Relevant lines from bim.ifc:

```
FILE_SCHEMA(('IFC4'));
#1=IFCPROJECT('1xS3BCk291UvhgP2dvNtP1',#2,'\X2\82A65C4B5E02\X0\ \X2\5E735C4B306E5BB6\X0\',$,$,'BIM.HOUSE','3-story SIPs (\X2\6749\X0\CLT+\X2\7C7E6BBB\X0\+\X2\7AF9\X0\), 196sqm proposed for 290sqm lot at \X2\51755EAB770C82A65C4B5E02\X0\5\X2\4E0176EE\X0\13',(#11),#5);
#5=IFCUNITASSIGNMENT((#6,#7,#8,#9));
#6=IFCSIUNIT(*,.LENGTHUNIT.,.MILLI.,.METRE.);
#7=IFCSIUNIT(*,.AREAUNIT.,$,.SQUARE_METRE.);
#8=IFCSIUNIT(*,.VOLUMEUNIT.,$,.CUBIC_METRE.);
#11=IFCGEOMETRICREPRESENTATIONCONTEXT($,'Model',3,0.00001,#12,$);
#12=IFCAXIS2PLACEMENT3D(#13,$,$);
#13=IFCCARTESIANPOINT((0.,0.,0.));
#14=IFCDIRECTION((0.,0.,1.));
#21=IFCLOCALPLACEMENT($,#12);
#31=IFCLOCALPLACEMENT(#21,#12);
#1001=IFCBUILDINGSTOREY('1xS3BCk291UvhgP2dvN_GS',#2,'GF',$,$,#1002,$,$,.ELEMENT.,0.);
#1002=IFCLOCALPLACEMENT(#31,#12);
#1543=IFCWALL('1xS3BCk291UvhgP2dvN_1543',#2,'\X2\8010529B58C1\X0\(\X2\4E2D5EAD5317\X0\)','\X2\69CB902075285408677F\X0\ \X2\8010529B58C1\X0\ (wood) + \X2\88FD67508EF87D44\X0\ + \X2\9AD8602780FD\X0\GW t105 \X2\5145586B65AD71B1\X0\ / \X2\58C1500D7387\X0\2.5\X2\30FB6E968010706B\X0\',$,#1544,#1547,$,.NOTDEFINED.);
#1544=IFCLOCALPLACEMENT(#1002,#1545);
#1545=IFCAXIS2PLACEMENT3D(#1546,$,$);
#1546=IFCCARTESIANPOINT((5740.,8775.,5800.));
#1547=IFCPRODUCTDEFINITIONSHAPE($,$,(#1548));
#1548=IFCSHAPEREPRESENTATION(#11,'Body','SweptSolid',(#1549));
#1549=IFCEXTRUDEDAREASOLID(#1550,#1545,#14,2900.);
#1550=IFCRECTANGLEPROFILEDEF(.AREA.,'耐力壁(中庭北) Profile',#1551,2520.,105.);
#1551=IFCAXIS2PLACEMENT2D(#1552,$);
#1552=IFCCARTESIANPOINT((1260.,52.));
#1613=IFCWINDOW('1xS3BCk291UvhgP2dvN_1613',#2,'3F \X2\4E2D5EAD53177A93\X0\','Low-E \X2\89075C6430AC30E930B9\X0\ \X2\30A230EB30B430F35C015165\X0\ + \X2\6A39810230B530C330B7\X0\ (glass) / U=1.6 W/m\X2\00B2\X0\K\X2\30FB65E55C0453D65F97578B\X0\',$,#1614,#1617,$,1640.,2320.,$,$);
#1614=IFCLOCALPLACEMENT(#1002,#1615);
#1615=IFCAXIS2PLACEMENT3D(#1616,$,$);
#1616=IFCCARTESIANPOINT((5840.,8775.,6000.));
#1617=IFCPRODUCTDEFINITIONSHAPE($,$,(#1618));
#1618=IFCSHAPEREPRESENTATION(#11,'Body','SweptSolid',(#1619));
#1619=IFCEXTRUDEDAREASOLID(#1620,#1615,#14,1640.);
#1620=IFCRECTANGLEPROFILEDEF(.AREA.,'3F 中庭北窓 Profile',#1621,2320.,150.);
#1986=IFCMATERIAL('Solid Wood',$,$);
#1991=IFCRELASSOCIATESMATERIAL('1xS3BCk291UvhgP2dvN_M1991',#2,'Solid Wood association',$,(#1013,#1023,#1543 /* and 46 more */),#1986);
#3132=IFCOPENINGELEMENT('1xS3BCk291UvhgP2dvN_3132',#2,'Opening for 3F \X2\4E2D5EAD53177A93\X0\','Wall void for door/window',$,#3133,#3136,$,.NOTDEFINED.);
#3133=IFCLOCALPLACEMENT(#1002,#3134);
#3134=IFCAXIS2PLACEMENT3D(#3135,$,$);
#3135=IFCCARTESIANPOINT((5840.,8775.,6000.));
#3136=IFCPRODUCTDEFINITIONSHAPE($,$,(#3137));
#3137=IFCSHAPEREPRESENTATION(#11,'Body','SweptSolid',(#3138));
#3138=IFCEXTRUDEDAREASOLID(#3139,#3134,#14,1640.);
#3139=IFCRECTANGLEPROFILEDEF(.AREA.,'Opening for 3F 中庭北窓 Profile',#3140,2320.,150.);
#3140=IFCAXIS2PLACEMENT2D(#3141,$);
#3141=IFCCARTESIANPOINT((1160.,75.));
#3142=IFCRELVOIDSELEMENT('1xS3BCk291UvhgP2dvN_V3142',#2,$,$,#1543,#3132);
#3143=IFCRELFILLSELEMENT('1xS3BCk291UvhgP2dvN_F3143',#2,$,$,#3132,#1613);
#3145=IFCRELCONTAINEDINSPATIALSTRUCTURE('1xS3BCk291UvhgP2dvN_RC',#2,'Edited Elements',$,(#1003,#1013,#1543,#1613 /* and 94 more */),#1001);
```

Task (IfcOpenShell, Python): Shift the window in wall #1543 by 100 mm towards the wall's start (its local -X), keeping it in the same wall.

```python
import ifcopenshell
import ifcopenshell.api.geometry
import ifcopenshell.util.placement
import ifcopenshell.util.unit

model = ifcopenshell.open("bim.ifc")
unit_scale = ifcopenshell.util.unit.calculate_unit_scale(model)

window = model.by_guid("1xS3BCk291UvhgP2dvN_1613")
opening = window.FillsVoids[0].RelatingOpeningElement
wall = opening.VoidsElements[0].RelatingBuildingElement

wall_matrix = ifcopenshell.util.placement.get_local_placement(wall.ObjectPlacement)
shift = wall_matrix[:3, 0] * -0.1 / unit_scale
before = ifcopenshell.util.placement.get_local_placement(window.ObjectPlacement)[:3, 3].copy()

# The window is not placed relative to its opening, so move both.
for product in (opening, window):
    matrix = ifcopenshell.util.placement.get_local_placement(product.ObjectPlacement)
    matrix[:3, 3] += shift
    ifcopenshell.api.geometry.edit_object_placement(model, product=product, matrix=matrix, is_si=False)

after = ifcopenshell.util.placement.get_local_placement(window.ObjectPlacement)[:3, 3]
print("window moved by", (after - before).round(3) + 0.0)

model.write("bim_edited.ifc")
```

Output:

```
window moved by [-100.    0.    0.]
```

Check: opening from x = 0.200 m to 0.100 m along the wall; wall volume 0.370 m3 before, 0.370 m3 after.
